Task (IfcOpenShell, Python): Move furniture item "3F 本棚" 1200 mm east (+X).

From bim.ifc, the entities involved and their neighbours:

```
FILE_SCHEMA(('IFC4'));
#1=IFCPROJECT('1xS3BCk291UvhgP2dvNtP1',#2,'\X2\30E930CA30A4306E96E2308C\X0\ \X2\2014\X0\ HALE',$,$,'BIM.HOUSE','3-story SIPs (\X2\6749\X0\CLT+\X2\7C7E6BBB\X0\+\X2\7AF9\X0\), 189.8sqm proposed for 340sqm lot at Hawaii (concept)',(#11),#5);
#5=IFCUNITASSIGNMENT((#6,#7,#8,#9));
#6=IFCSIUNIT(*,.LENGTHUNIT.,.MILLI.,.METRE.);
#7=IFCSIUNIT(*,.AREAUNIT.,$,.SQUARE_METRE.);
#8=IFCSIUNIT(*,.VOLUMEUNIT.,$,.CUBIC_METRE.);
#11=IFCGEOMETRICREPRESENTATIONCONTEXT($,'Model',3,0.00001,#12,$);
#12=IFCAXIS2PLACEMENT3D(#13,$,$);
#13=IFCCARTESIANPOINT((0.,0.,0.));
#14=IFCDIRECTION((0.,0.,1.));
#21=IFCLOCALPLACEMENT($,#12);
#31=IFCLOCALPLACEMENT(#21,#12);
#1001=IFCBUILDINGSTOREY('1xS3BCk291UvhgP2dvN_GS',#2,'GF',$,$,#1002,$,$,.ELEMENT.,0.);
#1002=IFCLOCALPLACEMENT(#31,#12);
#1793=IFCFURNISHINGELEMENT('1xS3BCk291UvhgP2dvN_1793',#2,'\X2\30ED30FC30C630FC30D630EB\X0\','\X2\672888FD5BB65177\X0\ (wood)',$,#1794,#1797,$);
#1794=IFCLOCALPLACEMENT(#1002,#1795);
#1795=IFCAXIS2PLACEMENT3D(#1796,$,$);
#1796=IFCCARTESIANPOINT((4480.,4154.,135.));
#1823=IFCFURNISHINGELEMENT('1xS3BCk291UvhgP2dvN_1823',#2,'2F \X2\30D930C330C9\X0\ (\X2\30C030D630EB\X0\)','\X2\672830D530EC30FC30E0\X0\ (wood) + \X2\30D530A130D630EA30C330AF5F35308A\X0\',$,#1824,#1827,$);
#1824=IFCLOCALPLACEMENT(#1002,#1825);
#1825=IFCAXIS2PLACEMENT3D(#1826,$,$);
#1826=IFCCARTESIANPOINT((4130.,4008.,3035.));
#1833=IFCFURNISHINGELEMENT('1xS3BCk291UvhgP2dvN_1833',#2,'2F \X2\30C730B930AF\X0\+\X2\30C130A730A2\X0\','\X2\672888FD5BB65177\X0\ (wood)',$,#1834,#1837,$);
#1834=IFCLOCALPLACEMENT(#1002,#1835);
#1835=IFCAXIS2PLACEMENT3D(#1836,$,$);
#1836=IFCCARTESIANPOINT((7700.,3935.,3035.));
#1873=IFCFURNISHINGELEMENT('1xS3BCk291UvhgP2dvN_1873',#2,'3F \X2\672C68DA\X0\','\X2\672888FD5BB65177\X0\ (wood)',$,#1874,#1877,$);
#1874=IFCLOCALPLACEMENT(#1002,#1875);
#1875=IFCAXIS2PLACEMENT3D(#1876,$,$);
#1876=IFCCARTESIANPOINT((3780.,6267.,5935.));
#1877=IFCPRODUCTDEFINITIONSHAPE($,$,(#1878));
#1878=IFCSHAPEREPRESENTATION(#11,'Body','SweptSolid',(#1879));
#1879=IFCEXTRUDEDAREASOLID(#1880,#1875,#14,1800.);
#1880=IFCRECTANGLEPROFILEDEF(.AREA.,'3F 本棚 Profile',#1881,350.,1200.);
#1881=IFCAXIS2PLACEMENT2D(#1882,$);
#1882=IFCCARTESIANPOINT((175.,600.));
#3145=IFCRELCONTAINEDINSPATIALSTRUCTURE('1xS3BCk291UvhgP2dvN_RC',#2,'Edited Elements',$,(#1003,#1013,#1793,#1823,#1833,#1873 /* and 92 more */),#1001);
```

```python
import ifcopenshell
import ifcopenshell.api.geometry
import ifcopenshell.util.placement

model = ifcopenshell.open("bim.ifc")

item = model.by_guid("1xS3BCk291UvhgP2dvN_1873")
matrix = ifcopenshell.util.placement.get_local_placement(item.ObjectPlacement)
matrix[0, 3] += 1200.0
ifcopenshell.api.geometry.edit_object_placement(model, product=item, matrix=matrix, is_si=False)

print(ifcopenshell.util.placement.get_local_placement(item.ObjectPlacement).round(3) + 0.0)

model.write("bim_v2.ifc")
```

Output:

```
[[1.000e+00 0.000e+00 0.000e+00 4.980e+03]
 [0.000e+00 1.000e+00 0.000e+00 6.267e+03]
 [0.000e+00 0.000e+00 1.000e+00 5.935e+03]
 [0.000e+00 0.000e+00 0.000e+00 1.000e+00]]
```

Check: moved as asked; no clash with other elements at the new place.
